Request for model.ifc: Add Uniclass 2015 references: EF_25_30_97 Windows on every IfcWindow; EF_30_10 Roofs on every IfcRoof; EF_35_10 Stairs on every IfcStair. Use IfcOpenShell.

First a look at what the model holds.

```python
import ifcopenshell

model = ifcopenshell.open("model.ifc")
print(model.schema)
print("classifications:", [c.Name for c in model.by_type("IfcClassification")])
for ifc_class in ("IfcDoor", "IfcRoof", "IfcStair", "IfcWall", "IfcWindow"):
    print(ifc_class, len(model.by_type(ifc_class)))
```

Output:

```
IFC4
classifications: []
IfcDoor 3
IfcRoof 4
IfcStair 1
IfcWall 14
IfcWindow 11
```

```python
import ifcopenshell
import ifcopenshell.api.classification

model = ifcopenshell.open("model.ifc")

system = ifcopenshell.api.classification.add_classification(model, classification="Uniclass 2015")

codes = {
    "IfcWindow": ("EF_25_30_97", "Windows"),
    "IfcRoof": ("EF_30_10", "Roofs"),
    "IfcStair": ("EF_35_10", "Stairs"),
}
for ifc_class, (code, name) in codes.items():
    products = model.by_type(ifc_class)
    ifcopenshell.api.classification.add_reference(
        model, products=products, classification=system, identification=code, name=name
    )
    print(code, len(products))

model.write("model-out.ifc")
```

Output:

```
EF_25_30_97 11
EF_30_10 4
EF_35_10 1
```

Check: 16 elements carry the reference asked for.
